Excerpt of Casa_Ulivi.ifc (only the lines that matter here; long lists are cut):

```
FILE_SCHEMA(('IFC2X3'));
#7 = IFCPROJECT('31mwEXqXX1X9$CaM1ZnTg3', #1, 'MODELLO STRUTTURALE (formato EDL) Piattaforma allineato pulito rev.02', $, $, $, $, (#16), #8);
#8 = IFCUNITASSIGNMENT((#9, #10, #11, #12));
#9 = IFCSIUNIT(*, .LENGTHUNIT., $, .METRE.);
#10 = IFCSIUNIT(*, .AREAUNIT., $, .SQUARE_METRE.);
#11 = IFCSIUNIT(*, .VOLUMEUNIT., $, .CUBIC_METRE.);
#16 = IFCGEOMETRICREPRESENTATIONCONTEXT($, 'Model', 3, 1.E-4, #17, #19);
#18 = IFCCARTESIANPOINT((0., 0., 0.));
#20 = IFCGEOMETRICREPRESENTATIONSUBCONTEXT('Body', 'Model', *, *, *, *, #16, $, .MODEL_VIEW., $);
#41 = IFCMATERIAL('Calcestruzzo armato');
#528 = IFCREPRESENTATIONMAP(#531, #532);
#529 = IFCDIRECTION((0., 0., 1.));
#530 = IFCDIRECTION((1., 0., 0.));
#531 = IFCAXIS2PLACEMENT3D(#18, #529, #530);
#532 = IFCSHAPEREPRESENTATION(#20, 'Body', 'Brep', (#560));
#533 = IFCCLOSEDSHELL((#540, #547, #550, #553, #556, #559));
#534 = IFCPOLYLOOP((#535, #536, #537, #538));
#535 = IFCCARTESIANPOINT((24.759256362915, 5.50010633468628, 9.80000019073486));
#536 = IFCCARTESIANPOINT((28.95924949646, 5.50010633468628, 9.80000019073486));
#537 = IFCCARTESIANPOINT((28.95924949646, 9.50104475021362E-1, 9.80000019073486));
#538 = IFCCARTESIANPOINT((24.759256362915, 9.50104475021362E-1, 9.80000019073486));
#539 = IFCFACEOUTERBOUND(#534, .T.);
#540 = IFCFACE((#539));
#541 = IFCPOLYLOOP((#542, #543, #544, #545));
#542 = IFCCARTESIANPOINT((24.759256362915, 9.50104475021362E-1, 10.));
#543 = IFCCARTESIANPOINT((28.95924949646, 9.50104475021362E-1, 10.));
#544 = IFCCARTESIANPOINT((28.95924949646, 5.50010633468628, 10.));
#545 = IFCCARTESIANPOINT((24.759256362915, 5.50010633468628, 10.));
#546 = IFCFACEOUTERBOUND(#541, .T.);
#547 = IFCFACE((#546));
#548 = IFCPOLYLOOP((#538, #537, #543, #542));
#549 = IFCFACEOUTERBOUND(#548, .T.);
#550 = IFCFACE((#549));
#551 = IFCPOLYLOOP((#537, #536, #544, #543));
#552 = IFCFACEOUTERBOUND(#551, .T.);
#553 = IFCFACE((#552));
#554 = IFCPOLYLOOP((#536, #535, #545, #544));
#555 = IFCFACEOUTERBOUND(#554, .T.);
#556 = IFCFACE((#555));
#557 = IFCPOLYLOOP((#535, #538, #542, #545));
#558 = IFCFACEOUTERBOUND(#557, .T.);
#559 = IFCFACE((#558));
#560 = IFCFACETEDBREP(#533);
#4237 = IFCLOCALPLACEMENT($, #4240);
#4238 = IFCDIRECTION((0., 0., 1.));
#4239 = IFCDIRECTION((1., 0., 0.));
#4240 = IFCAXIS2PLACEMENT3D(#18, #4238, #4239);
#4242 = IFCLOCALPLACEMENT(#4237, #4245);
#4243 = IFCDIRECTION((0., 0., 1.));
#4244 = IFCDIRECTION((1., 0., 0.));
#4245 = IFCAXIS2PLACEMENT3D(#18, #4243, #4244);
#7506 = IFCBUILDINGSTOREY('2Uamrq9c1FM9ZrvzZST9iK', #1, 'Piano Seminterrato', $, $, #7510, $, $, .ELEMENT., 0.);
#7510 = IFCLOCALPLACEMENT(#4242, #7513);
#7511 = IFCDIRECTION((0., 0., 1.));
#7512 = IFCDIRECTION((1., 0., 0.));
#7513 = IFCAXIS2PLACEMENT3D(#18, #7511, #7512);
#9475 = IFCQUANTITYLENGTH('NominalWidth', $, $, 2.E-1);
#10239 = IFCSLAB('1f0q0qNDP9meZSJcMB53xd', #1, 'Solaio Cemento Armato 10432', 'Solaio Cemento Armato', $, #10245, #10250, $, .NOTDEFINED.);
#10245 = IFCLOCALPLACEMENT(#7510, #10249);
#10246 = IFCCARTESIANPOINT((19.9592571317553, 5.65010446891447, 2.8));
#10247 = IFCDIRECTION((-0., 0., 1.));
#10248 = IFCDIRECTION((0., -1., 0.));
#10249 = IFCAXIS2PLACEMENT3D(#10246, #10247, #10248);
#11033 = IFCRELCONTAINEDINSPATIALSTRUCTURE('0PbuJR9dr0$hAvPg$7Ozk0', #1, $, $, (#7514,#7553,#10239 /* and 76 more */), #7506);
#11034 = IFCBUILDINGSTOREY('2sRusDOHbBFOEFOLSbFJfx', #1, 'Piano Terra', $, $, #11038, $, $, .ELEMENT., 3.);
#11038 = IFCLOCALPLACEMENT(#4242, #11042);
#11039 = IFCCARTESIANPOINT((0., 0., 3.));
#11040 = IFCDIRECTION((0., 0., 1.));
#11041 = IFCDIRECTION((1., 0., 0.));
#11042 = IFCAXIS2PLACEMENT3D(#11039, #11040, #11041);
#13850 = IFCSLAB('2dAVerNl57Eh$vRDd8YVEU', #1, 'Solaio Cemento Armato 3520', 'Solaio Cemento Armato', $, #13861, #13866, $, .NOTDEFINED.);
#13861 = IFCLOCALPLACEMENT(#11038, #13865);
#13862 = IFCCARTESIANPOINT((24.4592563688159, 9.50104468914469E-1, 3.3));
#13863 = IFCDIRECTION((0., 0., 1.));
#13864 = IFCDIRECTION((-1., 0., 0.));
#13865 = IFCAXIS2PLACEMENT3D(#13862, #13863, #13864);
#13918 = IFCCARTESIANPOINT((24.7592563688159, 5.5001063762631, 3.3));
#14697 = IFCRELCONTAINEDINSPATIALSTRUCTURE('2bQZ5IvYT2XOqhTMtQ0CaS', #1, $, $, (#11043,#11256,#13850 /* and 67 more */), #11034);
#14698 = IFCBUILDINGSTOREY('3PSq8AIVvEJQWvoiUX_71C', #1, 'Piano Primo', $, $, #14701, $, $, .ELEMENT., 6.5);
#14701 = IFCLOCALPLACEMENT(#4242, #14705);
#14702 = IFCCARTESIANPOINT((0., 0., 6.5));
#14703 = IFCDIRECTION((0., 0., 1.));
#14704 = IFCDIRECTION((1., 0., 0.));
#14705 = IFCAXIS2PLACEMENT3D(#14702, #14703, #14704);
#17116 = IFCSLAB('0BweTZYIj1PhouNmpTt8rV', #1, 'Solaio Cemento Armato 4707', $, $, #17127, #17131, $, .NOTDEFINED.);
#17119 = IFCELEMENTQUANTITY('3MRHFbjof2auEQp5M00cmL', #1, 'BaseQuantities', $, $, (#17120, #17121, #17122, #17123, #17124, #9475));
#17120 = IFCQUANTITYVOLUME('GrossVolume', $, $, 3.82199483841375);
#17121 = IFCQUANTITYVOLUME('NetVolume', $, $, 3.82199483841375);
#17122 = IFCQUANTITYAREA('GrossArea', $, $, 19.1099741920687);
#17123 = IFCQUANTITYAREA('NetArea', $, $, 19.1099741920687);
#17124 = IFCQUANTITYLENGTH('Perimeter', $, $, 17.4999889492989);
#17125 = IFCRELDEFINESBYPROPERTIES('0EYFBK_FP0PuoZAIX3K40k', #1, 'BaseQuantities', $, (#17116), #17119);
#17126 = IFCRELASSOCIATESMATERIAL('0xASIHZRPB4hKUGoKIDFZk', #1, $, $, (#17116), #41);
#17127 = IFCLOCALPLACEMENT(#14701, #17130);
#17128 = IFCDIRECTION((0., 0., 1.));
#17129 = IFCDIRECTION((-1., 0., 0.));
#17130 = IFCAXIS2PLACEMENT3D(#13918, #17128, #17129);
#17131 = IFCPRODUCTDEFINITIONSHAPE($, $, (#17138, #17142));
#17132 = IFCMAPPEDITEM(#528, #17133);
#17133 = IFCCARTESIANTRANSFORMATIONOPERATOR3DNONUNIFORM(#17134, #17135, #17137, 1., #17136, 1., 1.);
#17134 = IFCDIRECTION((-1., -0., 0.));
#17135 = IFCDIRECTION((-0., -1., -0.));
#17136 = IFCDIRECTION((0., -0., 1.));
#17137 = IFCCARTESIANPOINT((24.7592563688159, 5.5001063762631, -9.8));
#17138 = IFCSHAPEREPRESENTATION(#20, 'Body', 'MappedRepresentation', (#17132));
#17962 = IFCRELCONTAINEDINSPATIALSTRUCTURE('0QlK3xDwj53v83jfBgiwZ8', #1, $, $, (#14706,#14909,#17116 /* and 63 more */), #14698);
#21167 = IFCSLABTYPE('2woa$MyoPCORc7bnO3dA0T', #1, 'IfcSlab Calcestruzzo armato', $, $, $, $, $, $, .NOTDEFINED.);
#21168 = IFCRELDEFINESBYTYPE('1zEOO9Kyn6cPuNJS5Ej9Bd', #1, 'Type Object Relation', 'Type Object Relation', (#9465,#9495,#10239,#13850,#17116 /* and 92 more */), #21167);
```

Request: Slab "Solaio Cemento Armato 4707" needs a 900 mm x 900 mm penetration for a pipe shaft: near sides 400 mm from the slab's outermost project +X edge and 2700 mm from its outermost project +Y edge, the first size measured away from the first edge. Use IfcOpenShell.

```python
import numpy as np
import ifcopenshell
import ifcopenshell.api.feature
import ifcopenshell.api.geometry
import ifcopenshell.api.pset
import ifcopenshell.api.root
import ifcopenshell.geom
import ifcopenshell.util.element
import ifcopenshell.util.placement
import ifcopenshell.util.representation
import ifcopenshell.util.shape
import ifcopenshell.util.unit

model = ifcopenshell.open("Casa_Ulivi.ifc")
unit_scale = ifcopenshell.util.unit.calculate_unit_scale(model)
area_scale = ifcopenshell.util.unit.calculate_unit_scale(model, "AREAUNIT")
volume_scale = ifcopenshell.util.unit.calculate_unit_scale(model, "VOLUMEUNIT")
settings = ifcopenshell.geom.settings()


def volume(element):
    """Net volume in cubic metres, openings subtracted."""
    shape = ifcopenshell.geom.create_shape(settings, element)
    return ifcopenshell.util.shape.get_volume(shape.geometry)


slab = model.by_guid("0BweTZYIj1PhouNmpTt8rV")
before = volume(slab)

# Extent in the slab's own axes, in metres. The edges named are its -X and -Y sides.
slab_shape = ifcopenshell.geom.create_shape(settings, slab)
vertices = ifcopenshell.util.shape.get_vertices(slab_shape.geometry)
x_min, y_min, bottom = vertices.min(axis=0)
top = vertices[:, 2].max()

opening = ifcopenshell.api.root.create_entity(model, ifc_class="IfcOpeningElement", name="Pipe shaft opening")
context = ifcopenshell.util.representation.get_context(model, "Model", "Body", "MODEL_VIEW")
width, depth = 0.9, 0.9
outline = [(0.0, 0.0), (width, 0.0), (width, depth), (0.0, depth), (0.0, 0.0)]
# Overshoot both faces by 50 mm so the cut is clean.
shape = ifcopenshell.api.geometry.add_slab_representation(
    model, context=context, depth=top - bottom + 0.1, polyline=outline
)
ifcopenshell.api.geometry.assign_representation(model, product=opening, representation=shape)

matrix = ifcopenshell.util.placement.get_local_placement(slab.ObjectPlacement)
matrix[:, 3] = matrix @ np.append(np.array([x_min + 0.4, y_min + 2.7, bottom - 0.05]) / unit_scale, 1.0)
ifcopenshell.api.geometry.edit_object_placement(model, product=opening, matrix=matrix, is_si=False)
ifcopenshell.api.feature.add_feature(model, feature=opening, element=slab)

after = volume(slab)

# Update the slab's stored quantities.
qto = model.by_id(ifcopenshell.util.element.get_pset(slab, "BaseQuantities", should_inherit=False)["id"])
ifcopenshell.api.pset.edit_qto(model, qto=qto, properties={
    "NetVolume": after / volume_scale,
    "NetArea": after / (top - bottom) / area_scale,
})

print(f"slab volume {before:.3f} -> {after:.3f} m3")

model.write("Casa_Ulivi-out.ifc")
```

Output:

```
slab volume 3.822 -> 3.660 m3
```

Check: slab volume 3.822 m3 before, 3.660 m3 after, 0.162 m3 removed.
